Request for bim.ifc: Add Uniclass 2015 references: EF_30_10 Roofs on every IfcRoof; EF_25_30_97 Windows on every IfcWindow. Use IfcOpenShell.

First a look at what the model holds.

```python
import ifcopenshell

model = ifcopenshell.open("bim.ifc")
print(model.schema)
print("classifications:", [c.Name for c in model.by_type("IfcClassification")])
for ifc_class in ("IfcDoor", "IfcRoof", "IfcStair", "IfcWall", "IfcWindow"):
    print(ifc_class, len(model.by_type(ifc_class)))
```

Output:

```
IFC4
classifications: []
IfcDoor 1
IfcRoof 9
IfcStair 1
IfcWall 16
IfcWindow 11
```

```python
import ifcopenshell
import ifcopenshell.api.classification

model = ifcopenshell.open("bim.ifc")

system = ifcopenshell.api.classification.add_classification(model, classification="Uniclass 2015")

codes = {
    "IfcRoof": ("EF_30_10", "Roofs"),
    "IfcWindow": ("EF_25_30_97", "Windows"),
}
for ifc_class, (code, name) in codes.items():
    products = model.by_type(ifc_class)
    ifcopenshell.api.classification.add_reference(
        model, products=products, classification=system, identification=code, name=name
    )
    print(code, len(products))

model.write("bim_edited.ifc")
```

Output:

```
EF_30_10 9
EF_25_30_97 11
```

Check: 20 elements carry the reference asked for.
